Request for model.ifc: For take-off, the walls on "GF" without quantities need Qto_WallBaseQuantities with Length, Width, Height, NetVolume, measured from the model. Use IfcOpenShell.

First a look at what the model holds.

```python
import ifcopenshell
import ifcopenshell.util.element
import ifcopenshell.util.unit

model = ifcopenshell.open("model.ifc")
print(model.schema)
for unit_type in ("LENGTHUNIT", "AREAUNIT", "VOLUMEUNIT"):
    print(unit_type, ifcopenshell.util.unit.calculate_unit_scale(model, unit_type))
storey = next(s for s in model.by_type("IfcBuildingStorey") if s.Name == "GF")
walls = [e for e in ifcopenshell.util.element.get_decomposition(storey) if e.is_a("IfcWall")]
for e in sorted(walls, key=lambda e: e.id()):
    print(e.id(), e.is_a(), e.Name, list(ifcopenshell.util.element.get_psets(e, qtos_only=True)), sep=" | ")
```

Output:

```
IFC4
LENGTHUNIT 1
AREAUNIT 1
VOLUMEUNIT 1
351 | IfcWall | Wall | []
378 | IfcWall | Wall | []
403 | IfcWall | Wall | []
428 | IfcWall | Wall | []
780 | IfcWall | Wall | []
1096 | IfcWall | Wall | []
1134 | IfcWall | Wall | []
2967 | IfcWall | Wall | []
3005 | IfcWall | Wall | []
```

```python
import ifcopenshell
import ifcopenshell.api.pset
import ifcopenshell.geom
import ifcopenshell.util.element
import ifcopenshell.util.shape
import ifcopenshell.util.unit

model = ifcopenshell.open("model.ifc")
unit_scale = ifcopenshell.util.unit.calculate_unit_scale(model)
volume_scale = ifcopenshell.util.unit.calculate_unit_scale(model, "VOLUMEUNIT")
settings = ifcopenshell.geom.settings()

storey = next(s for s in model.by_type("IfcBuildingStorey") if s.Name == "GF")
walls = [e for e in ifcopenshell.util.element.get_decomposition(storey) if e.is_a("IfcWall")]

for e in sorted(walls, key=lambda e: e.id()):
    if ifcopenshell.util.element.get_psets(e, qtos_only=True, should_inherit=False):
        continue
    # Geometry comes back in metres, in the element's own axes.
    shape = ifcopenshell.geom.create_shape(settings, e)
    values = {
        "Length": ifcopenshell.util.shape.get_x(shape.geometry) / unit_scale,
        "Width": ifcopenshell.util.shape.get_y(shape.geometry) / unit_scale,
        "Height": ifcopenshell.util.shape.get_z(shape.geometry) / unit_scale,
        "NetVolume": ifcopenshell.util.shape.get_volume(shape.geometry) / volume_scale,
    }
    qto = ifcopenshell.api.pset.add_qto(model, product=e, name="Qto_WallBaseQuantities")
    ifcopenshell.api.pset.edit_qto(model, qto=qto, properties=values)
    print(e.id(), {k: round(v, 3) for k, v in values.items()})

model.write("model_v2.ifc")
```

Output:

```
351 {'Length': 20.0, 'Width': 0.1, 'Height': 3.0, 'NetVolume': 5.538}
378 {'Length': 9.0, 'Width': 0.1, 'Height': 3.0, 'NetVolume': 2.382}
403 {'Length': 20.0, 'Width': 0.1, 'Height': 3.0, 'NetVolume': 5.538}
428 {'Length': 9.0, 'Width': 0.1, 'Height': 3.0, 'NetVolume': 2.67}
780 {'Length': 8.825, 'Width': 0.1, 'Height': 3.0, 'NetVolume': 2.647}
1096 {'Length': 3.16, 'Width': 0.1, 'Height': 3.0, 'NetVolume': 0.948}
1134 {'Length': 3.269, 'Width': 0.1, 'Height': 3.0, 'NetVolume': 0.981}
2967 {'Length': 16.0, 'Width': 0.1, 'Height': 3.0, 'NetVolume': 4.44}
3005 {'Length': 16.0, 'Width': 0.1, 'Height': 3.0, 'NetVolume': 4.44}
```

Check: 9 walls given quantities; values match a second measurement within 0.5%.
